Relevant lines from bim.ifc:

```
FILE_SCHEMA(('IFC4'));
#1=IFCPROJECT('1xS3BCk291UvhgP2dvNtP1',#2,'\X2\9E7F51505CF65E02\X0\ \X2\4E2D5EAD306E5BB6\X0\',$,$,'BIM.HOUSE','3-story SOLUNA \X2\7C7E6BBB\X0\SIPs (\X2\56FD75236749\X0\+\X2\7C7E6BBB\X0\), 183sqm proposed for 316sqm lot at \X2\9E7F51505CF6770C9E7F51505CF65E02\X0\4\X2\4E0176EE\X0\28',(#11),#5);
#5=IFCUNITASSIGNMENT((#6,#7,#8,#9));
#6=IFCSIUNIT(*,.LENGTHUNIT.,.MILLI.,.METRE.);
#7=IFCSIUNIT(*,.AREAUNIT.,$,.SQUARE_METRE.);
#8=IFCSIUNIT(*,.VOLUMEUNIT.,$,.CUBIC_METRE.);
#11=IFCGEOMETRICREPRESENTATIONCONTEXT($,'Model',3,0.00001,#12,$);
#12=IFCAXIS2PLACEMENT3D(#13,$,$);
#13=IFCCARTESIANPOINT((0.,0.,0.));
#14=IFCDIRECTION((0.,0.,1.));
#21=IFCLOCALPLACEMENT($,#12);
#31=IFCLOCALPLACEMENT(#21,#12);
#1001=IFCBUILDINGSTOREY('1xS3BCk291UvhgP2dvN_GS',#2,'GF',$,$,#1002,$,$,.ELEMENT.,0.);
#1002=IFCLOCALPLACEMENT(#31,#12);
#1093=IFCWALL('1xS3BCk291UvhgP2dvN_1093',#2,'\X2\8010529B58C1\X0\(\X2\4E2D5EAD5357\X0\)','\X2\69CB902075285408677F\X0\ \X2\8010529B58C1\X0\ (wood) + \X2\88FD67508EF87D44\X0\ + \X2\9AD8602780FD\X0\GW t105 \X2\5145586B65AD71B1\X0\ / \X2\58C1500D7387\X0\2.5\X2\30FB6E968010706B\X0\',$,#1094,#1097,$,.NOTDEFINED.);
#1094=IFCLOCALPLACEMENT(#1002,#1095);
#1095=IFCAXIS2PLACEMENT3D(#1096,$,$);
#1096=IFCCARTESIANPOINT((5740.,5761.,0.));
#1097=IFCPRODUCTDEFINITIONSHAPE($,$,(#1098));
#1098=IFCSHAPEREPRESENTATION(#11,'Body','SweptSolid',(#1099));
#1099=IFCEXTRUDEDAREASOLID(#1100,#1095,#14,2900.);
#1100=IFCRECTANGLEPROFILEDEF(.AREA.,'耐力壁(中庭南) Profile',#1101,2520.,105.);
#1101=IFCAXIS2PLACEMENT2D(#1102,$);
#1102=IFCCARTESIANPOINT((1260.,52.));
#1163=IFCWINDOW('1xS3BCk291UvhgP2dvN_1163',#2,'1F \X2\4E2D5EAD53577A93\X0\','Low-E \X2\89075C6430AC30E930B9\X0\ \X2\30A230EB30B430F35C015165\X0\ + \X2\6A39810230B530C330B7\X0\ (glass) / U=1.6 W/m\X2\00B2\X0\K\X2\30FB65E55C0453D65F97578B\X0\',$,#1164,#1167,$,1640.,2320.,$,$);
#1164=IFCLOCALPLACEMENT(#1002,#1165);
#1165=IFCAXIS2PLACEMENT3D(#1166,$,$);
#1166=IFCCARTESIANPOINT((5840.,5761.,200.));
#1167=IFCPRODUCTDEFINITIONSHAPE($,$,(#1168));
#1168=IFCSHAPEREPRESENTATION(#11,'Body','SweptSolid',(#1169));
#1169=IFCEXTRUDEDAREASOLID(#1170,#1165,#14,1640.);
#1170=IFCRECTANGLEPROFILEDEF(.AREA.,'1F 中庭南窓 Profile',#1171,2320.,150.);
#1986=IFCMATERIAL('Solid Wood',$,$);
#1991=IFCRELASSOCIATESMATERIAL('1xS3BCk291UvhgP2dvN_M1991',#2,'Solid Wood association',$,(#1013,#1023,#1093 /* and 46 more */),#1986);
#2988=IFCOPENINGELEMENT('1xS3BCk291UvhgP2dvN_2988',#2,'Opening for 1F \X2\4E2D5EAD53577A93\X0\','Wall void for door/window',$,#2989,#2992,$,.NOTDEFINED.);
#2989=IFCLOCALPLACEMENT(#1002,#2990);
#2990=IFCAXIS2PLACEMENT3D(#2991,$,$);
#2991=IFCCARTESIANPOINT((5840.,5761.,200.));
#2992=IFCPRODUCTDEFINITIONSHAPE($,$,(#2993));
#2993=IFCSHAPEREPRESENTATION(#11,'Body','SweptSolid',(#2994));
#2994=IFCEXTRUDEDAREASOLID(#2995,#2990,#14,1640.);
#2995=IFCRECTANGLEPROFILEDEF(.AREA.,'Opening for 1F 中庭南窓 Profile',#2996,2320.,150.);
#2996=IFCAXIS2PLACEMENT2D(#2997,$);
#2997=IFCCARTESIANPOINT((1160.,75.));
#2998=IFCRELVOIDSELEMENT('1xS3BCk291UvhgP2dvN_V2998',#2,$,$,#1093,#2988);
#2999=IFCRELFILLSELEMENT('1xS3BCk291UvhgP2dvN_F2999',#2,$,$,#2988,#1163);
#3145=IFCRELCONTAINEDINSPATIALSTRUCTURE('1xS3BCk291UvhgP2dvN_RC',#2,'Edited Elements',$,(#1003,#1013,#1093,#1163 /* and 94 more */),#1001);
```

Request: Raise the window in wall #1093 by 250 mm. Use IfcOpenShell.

```python
import numpy as np
import ifcopenshell
import ifcopenshell.api.geometry
import ifcopenshell.util.placement
import ifcopenshell.util.unit

model = ifcopenshell.open("bim.ifc")
unit_scale = ifcopenshell.util.unit.calculate_unit_scale(model)

window = model.by_id(1163)
opening = window.FillsVoids[0].RelatingOpeningElement
dz = 250.0

shift = np.array([0.0, 0.0, dz])
# The window is not placed relative to its opening, so move both.
for product in (opening, window):
    matrix = ifcopenshell.util.placement.get_local_placement(product.ObjectPlacement)
    matrix[:3, 3] += shift
    ifcopenshell.api.geometry.edit_object_placement(model, product=product, matrix=matrix, is_si=False)

print(f"moved by {dz * unit_scale:+.3f} m")

model.write("bim_rev.ifc")
```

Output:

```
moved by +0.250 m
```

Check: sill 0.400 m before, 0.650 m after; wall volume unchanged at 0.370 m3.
